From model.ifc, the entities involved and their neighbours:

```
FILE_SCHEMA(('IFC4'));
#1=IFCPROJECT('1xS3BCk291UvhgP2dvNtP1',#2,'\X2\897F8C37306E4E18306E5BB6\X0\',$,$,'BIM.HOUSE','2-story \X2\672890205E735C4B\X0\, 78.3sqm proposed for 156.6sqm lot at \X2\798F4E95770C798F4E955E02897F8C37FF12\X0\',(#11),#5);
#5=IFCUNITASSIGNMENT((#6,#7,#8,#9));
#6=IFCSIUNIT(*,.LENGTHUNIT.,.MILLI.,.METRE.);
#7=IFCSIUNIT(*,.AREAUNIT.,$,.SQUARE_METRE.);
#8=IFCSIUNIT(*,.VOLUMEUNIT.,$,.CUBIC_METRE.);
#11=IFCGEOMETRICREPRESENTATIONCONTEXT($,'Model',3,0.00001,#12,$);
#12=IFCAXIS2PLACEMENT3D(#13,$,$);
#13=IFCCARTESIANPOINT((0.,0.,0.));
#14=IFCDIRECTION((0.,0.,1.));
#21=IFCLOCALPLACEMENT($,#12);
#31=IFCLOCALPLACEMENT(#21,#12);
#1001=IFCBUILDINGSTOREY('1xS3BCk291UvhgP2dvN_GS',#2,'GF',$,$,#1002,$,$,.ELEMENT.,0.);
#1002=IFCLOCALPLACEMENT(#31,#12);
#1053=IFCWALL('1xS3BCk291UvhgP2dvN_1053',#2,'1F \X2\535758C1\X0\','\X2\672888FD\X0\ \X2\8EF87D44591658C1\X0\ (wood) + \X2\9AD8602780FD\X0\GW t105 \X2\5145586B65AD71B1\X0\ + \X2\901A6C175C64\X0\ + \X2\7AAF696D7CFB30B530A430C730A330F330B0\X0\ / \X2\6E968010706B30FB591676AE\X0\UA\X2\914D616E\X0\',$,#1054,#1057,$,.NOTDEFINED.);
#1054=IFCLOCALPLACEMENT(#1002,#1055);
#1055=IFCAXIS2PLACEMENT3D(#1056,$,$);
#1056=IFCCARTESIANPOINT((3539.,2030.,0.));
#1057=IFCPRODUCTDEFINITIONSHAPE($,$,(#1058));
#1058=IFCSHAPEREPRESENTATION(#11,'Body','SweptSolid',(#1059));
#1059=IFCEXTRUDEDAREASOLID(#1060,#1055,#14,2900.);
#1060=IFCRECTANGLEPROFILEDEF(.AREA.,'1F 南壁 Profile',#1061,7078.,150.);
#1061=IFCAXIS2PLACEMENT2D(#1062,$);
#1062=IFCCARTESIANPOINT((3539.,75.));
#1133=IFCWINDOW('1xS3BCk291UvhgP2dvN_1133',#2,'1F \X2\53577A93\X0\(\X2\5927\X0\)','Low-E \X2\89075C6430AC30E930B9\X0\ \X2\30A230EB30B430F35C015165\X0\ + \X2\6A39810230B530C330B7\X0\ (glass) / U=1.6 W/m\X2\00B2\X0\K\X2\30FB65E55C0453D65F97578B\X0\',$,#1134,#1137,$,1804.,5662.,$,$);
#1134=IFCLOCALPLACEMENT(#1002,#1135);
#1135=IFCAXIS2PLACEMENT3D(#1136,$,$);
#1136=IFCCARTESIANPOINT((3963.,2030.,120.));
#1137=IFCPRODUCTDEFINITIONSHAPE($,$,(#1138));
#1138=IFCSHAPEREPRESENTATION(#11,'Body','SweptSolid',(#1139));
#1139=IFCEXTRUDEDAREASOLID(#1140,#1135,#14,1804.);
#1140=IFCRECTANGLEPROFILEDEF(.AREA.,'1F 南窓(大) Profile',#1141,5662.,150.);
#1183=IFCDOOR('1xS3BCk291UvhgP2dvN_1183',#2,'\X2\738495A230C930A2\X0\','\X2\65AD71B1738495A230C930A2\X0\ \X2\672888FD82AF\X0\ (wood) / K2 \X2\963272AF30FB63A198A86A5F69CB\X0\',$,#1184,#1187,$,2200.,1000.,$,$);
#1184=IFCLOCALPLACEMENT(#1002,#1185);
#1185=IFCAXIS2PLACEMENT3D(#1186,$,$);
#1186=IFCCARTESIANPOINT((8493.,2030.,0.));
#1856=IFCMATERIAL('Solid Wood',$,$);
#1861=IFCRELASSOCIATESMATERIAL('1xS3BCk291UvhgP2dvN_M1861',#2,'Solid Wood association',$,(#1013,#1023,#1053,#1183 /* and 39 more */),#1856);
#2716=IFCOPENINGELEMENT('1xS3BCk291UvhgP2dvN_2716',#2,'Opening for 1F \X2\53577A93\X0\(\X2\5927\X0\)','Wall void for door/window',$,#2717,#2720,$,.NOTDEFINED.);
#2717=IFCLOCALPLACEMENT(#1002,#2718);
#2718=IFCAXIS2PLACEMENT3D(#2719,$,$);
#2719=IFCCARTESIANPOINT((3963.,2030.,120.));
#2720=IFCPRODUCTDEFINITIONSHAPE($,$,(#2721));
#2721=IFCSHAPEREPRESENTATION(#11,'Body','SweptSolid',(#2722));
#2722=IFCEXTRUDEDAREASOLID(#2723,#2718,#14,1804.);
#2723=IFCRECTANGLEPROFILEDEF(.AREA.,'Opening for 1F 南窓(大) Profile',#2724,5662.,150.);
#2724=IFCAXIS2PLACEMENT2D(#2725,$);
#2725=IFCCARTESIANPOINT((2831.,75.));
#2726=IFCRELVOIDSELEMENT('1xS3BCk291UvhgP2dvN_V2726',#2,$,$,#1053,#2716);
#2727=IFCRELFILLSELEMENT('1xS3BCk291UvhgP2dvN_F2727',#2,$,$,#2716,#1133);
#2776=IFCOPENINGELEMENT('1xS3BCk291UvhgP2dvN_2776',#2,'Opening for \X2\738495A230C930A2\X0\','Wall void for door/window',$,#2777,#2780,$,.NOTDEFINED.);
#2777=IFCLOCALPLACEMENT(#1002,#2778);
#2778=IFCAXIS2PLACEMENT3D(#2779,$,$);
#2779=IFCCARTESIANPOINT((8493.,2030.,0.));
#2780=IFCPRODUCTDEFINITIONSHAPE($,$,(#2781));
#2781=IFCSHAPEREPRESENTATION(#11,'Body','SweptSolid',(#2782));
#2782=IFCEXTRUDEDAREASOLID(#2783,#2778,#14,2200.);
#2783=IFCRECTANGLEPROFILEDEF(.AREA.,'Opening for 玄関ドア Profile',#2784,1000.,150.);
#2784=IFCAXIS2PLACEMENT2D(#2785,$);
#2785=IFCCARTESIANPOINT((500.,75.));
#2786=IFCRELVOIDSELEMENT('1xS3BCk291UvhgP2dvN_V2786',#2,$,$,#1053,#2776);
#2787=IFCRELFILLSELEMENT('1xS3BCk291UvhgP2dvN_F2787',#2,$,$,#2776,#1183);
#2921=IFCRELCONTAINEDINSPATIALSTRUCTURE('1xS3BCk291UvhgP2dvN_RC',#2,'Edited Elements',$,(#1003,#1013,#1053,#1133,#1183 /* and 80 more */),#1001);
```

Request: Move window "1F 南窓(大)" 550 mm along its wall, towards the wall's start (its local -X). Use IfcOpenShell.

```python
import ifcopenshell
import ifcopenshell.api.geometry
import ifcopenshell.util.placement

model = ifcopenshell.open("model.ifc")

window = model.by_guid("1xS3BCk291UvhgP2dvN_1133")
opening = window.FillsVoids[0].RelatingOpeningElement
wall = opening.VoidsElements[0].RelatingBuildingElement

wall_matrix = ifcopenshell.util.placement.get_local_placement(wall.ObjectPlacement)
shift = wall_matrix[:3, 0] * -550.0
before = ifcopenshell.util.placement.get_local_placement(window.ObjectPlacement)[:3, 3].copy()

# The window is not placed relative to its opening, so move both.
for product in (opening, window):
    matrix = ifcopenshell.util.placement.get_local_placement(product.ObjectPlacement)
    matrix[:3, 3] += shift
    ifcopenshell.api.geometry.edit_object_placement(model, product=product, matrix=matrix, is_si=False)

after = ifcopenshell.util.placement.get_local_placement(window.ObjectPlacement)[:3, 3]
print("window moved by", (after - before).round(3) + 0.0)

model.write("model_updated.ifc")
```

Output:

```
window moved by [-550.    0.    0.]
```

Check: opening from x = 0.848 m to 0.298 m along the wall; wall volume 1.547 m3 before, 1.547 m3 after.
